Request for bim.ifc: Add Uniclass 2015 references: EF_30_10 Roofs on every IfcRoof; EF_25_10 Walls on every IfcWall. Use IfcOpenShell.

First a look at what the model holds.

```python
import ifcopenshell

model = ifcopenshell.open("bim.ifc")
print(model.schema)
print("classifications:", [c.Name for c in model.by_type("IfcClassification")])
for ifc_class in ("IfcDoor", "IfcRoof", "IfcStair", "IfcWall", "IfcWindow"):
    print(ifc_class, len(model.by_type(ifc_class)))
```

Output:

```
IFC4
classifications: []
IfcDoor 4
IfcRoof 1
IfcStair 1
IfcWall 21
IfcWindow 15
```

```python
import ifcopenshell
import ifcopenshell.api.classification

model = ifcopenshell.open("bim.ifc")

system = ifcopenshell.api.classification.add_classification(model, classification="Uniclass 2015")

codes = {
    "IfcRoof": ("EF_30_10", "Roofs"),
    "IfcWall": ("EF_25_10", "Walls"),
}
for ifc_class, (code, name) in codes.items():
    products = model.by_type(ifc_class)
    ifcopenshell.api.classification.add_reference(
        model, products=products, classification=system, identification=code, name=name
    )
    print(code, len(products))

model.write("bim-out.ifc")
```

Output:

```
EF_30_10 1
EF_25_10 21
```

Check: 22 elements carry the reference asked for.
